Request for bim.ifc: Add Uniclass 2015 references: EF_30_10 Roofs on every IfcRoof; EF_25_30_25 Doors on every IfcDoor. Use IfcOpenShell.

First a look at what the model holds.

```python
import ifcopenshell

model = ifcopenshell.open("bim.ifc")
print(model.schema)
print("classifications:", [c.Name for c in model.by_type("IfcClassification")])
for ifc_class in ("IfcDoor", "IfcRoof", "IfcStair", "IfcWall", "IfcWindow"):
    print(ifc_class, len(model.by_type(ifc_class)))
```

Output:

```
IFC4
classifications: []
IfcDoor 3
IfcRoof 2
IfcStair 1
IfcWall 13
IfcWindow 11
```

```python
import ifcopenshell
import ifcopenshell.api.classification

model = ifcopenshell.open("bim.ifc")

system = ifcopenshell.api.classification.add_classification(model, classification="Uniclass 2015")

codes = {
    "IfcRoof": ("EF_30_10", "Roofs"),
    "IfcDoor": ("EF_25_30_25", "Doors"),
}
for ifc_class, (code, name) in codes.items():
    products = model.by_type(ifc_class)
    ifcopenshell.api.classification.add_reference(
        model, products=products, classification=system, identification=code, name=name
    )
    print(code, len(products))

model.write("bim_edited.ifc")
```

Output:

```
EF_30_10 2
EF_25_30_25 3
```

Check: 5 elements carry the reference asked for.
